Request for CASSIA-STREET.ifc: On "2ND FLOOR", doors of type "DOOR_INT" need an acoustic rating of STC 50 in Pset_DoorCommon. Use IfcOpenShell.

First a look at what the model holds.

```python
import ifcopenshell
import ifcopenshell.util.element

model = ifcopenshell.open("CASSIA-STREET.ifc")
print(model.schema)
storey = next(s for s in model.by_type("IfcBuildingStorey") if s.Name == "2ND FLOOR")
doors = [e for e in ifcopenshell.util.element.get_decomposition(storey) if e.is_a("IfcDoor")]
seen = {}
for e in doors:
    element_type = ifcopenshell.util.element.get_type(e)
    key = (element_type.Name if element_type != e and element_type else None, ifcopenshell.util.element.get_pset(e, "Pset_DoorCommon", "AcousticRating"))
    seen[key] = seen.get(key, 0) + 1
for (name, value), count in sorted(seen.items(), key=str):
    print(count, "x", name, "|", value)
```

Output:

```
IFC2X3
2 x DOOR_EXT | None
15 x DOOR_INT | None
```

```python
import ifcopenshell
import ifcopenshell.api.pset
import ifcopenshell.util.element

model = ifcopenshell.open("CASSIA-STREET.ifc")

storey = next(s for s in model.by_type("IfcBuildingStorey") if s.Name == "2ND FLOOR")
doors = [e for e in ifcopenshell.util.element.get_decomposition(storey) if e.is_a("IfcDoor")]

count = 0
for e in doors:
    element_type = ifcopenshell.util.element.get_type(e)
    if element_type in (None, e) or element_type.Name != "DOOR_INT":
        continue
    # add_pset returns the element's existing set when there is one.
    pset = ifcopenshell.api.pset.add_pset(model, product=e, name="Pset_DoorCommon")
    ifcopenshell.api.pset.edit_pset(model, pset=pset, properties={"AcousticRating": "STC 50"})
    count += 1

print(count, "doors updated")

model.write("CASSIA-STREET_v2.ifc")
```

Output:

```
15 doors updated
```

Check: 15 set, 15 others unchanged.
